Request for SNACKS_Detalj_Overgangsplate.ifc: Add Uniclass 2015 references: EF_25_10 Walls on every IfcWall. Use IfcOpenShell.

First a look at what the model holds.

```python
import ifcopenshell

model = ifcopenshell.open("SNACKS_Detalj_Overgangsplate.ifc")
print(model.schema)
print("classifications:", [c.Name for c in model.by_type("IfcClassification")])
for ifc_class in ("IfcDoor", "IfcRoof", "IfcStair", "IfcWall", "IfcWindow"):
    print(ifc_class, len(model.by_type(ifc_class)))
```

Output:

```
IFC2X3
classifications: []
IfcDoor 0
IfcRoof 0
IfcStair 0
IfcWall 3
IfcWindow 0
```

```python
import ifcopenshell
import ifcopenshell.api.classification

model = ifcopenshell.open("SNACKS_Detalj_Overgangsplate.ifc")

# IFC2X3 requires Source and Edition and has no link from the project to the system.
system = model.create_entity("IfcClassification", Source="NBS", Edition="2015", Name="Uniclass 2015")

codes = {
    "IfcWall": ("EF_25_10", "Walls"),
}
for ifc_class, (code, name) in codes.items():
    products = model.by_type(ifc_class)
    ifcopenshell.api.classification.add_reference(
        model, products=products, classification=system, identification=code, name=name
    )
    print(code, len(products))

model.write("SNACKS_Detalj_Overgangsplate_edited.ifc")
```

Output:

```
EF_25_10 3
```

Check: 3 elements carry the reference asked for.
